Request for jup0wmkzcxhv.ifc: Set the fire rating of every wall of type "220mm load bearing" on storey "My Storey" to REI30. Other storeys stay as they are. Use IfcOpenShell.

First a look at what the model holds.

```python
import ifcopenshell
import ifcopenshell.util.element

model = ifcopenshell.open("jup0wmkzcxhv.ifc")
print(model.schema)
storey = next(s for s in model.by_type("IfcBuildingStorey") if s.Name == "My Storey")
walls = [e for e in ifcopenshell.util.element.get_decomposition(storey) if e.is_a("IfcWall")]
seen = {}
for e in walls:
    element_type = ifcopenshell.util.element.get_type(e)
    key = (element_type.Name if element_type != e and element_type else None, ifcopenshell.util.element.get_pset(e, "Pset_WallCommon", "FireRating"))
    seen[key] = seen.get(key, 0) + 1
for (name, value), count in sorted(seen.items(), key=str):
    print(count, "x", name, "|", value)
```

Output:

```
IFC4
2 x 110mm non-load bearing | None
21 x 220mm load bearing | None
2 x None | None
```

```python
import ifcopenshell
import ifcopenshell.api.pset
import ifcopenshell.util.element

model = ifcopenshell.open("jup0wmkzcxhv.ifc")

storey = next(s for s in model.by_type("IfcBuildingStorey") if s.Name == "My Storey")
walls = [e for e in ifcopenshell.util.element.get_decomposition(storey) if e.is_a("IfcWall")]

count = 0
for e in walls:
    element_type = ifcopenshell.util.element.get_type(e)
    if element_type in (None, e) or element_type.Name != "220mm load bearing":
        continue
    # add_pset returns the element's existing set when there is one.
    pset = ifcopenshell.api.pset.add_pset(model, product=e, name="Pset_WallCommon")
    ifcopenshell.api.pset.edit_pset(model, pset=pset, properties={"FireRating": "REI30"})
    count += 1

print(count, "walls updated")

model.write("jup0wmkzcxhv_updated.ifc")
```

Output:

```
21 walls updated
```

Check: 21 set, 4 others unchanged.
